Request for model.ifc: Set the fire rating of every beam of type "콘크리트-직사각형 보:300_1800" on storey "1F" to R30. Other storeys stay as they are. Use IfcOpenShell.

First a look at what the model holds.

```python
import ifcopenshell
import ifcopenshell.util.element

model = ifcopenshell.open("model.ifc")
print(model.schema)
storey = next(s for s in model.by_type("IfcBuildingStorey") if s.Name == "1F")
beams = [e for e in ifcopenshell.util.element.get_decomposition(storey) if e.is_a("IfcBeam")]
seen = {}
for e in beams:
    element_type = ifcopenshell.util.element.get_type(e)
    key = (element_type.Name if element_type != e and element_type else None, ifcopenshell.util.element.get_pset(e, "Pset_BeamCommon", "FireRating"))
    seen[key] = seen.get(key, 0) + 1
for (name, value), count in sorted(seen.items(), key=str):
    print(count, "x", name, "|", value)
```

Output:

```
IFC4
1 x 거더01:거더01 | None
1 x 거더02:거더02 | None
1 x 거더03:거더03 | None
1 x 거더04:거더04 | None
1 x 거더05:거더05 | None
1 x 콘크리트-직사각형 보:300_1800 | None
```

```python
import ifcopenshell
import ifcopenshell.api.pset
import ifcopenshell.util.element

model = ifcopenshell.open("model.ifc")

storey = next(s for s in model.by_type("IfcBuildingStorey") if s.Name == "1F")
beams = [e for e in ifcopenshell.util.element.get_decomposition(storey) if e.is_a("IfcBeam")]

count = 0
for e in beams:
    element_type = ifcopenshell.util.element.get_type(e)
    if element_type in (None, e) or element_type.Name != "콘크리트-직사각형 보:300_1800":
        continue
    # add_pset returns the element's existing set when there is one.
    pset = ifcopenshell.api.pset.add_pset(model, product=e, name="Pset_BeamCommon")
    ifcopenshell.api.pset.edit_pset(model, pset=pset, properties={"FireRating": "R30"})
    count += 1

print(count, "beams updated")

model.write("model-out.ifc")
```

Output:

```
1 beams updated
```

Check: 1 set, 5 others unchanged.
